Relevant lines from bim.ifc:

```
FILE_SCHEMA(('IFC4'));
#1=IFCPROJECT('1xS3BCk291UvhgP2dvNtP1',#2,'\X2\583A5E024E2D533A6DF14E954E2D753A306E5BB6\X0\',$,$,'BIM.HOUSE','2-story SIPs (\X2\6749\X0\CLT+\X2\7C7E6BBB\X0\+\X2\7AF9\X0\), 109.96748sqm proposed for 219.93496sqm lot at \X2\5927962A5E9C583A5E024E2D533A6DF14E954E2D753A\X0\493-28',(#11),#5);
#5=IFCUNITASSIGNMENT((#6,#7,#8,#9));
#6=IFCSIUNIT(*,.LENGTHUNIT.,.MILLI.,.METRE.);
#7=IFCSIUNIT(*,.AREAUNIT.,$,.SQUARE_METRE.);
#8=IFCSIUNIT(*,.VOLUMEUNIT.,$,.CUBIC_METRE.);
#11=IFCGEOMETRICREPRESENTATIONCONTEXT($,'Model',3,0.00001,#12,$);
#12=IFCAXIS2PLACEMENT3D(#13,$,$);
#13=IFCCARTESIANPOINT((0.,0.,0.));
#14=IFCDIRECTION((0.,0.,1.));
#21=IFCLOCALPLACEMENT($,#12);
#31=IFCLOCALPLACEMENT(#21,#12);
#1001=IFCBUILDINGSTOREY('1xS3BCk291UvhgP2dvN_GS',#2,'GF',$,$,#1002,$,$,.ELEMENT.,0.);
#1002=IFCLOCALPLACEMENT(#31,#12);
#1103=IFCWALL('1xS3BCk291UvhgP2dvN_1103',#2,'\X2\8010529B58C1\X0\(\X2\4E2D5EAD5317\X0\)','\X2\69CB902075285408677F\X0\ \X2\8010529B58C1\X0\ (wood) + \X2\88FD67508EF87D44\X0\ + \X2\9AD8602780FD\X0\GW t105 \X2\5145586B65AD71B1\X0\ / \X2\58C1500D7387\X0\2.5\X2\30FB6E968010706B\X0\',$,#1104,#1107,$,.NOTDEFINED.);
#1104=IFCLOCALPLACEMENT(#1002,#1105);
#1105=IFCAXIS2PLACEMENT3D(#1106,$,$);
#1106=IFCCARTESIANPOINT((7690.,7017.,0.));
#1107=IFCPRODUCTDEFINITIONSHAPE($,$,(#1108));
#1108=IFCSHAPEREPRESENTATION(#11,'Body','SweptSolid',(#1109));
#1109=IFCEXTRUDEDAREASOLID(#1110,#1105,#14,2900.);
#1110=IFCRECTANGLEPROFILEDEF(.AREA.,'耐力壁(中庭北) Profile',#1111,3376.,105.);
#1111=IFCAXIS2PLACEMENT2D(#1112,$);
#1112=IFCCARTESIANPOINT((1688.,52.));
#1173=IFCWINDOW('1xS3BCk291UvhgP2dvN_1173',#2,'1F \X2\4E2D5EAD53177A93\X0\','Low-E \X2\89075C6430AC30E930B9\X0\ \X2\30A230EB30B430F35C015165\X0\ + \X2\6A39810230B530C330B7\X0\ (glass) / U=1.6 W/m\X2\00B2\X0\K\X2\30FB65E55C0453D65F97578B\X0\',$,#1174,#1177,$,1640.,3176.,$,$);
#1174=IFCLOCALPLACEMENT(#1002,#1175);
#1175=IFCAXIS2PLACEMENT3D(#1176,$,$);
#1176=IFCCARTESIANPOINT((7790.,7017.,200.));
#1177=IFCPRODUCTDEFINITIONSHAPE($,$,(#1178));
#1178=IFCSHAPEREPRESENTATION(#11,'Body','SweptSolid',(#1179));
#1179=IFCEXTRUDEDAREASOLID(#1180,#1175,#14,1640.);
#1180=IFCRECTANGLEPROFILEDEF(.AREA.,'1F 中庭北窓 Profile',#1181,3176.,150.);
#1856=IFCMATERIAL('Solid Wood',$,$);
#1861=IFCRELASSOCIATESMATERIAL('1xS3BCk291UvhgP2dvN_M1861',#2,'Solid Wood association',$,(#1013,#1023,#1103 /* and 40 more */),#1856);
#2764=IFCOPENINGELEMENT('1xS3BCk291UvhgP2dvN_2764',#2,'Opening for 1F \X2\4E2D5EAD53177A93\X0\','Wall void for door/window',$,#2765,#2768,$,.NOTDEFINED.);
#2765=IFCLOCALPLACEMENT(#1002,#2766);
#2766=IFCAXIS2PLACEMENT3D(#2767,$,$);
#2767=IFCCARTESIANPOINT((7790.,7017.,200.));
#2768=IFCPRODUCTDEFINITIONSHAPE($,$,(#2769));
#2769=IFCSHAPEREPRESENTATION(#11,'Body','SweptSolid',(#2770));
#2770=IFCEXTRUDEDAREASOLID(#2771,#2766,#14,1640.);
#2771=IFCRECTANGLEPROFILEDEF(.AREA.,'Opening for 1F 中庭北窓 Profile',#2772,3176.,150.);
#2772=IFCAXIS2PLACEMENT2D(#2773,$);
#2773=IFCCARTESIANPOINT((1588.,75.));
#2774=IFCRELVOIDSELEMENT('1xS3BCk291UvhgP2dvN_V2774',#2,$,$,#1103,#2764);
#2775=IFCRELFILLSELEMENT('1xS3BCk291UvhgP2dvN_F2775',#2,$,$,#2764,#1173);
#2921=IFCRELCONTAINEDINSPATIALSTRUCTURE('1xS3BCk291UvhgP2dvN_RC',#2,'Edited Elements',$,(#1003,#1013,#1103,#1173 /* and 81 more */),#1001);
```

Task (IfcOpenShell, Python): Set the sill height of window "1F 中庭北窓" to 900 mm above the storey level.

```python
import numpy as np
import ifcopenshell
import ifcopenshell.api.geometry
import ifcopenshell.geom
import ifcopenshell.util.element
import ifcopenshell.util.placement
import ifcopenshell.util.shape
import ifcopenshell.util.unit

model = ifcopenshell.open("bim.ifc")
unit_scale = ifcopenshell.util.unit.calculate_unit_scale(model)

window = model.by_id(1173)
opening = window.FillsVoids[0].RelatingOpeningElement
storey = ifcopenshell.util.element.get_container(window, ifc_class="IfcBuildingStorey")
level = ifcopenshell.util.placement.get_local_placement(storey.ObjectPlacement)[2, 3]

# The opening's origin need not be at the sill, so measure its lowest point.
shape = ifcopenshell.geom.create_shape(ifcopenshell.geom.settings(), opening)
bottom = ifcopenshell.util.shape.get_shape_bottom_elevation(shape, shape.geometry) / unit_scale
dz = level + 0.9 / unit_scale - bottom

shift = np.array([0.0, 0.0, dz])
# The window is not placed relative to its opening, so move both.
for product in (opening, window):
    matrix = ifcopenshell.util.placement.get_local_placement(product.ObjectPlacement)
    matrix[:3, 3] += shift
    ifcopenshell.api.geometry.edit_object_placement(model, product=product, matrix=matrix, is_si=False)

print(f"moved by {dz * unit_scale:+.3f} m")

model.write("bim_v2.ifc")
```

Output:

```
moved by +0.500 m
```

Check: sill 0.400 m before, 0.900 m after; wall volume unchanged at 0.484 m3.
